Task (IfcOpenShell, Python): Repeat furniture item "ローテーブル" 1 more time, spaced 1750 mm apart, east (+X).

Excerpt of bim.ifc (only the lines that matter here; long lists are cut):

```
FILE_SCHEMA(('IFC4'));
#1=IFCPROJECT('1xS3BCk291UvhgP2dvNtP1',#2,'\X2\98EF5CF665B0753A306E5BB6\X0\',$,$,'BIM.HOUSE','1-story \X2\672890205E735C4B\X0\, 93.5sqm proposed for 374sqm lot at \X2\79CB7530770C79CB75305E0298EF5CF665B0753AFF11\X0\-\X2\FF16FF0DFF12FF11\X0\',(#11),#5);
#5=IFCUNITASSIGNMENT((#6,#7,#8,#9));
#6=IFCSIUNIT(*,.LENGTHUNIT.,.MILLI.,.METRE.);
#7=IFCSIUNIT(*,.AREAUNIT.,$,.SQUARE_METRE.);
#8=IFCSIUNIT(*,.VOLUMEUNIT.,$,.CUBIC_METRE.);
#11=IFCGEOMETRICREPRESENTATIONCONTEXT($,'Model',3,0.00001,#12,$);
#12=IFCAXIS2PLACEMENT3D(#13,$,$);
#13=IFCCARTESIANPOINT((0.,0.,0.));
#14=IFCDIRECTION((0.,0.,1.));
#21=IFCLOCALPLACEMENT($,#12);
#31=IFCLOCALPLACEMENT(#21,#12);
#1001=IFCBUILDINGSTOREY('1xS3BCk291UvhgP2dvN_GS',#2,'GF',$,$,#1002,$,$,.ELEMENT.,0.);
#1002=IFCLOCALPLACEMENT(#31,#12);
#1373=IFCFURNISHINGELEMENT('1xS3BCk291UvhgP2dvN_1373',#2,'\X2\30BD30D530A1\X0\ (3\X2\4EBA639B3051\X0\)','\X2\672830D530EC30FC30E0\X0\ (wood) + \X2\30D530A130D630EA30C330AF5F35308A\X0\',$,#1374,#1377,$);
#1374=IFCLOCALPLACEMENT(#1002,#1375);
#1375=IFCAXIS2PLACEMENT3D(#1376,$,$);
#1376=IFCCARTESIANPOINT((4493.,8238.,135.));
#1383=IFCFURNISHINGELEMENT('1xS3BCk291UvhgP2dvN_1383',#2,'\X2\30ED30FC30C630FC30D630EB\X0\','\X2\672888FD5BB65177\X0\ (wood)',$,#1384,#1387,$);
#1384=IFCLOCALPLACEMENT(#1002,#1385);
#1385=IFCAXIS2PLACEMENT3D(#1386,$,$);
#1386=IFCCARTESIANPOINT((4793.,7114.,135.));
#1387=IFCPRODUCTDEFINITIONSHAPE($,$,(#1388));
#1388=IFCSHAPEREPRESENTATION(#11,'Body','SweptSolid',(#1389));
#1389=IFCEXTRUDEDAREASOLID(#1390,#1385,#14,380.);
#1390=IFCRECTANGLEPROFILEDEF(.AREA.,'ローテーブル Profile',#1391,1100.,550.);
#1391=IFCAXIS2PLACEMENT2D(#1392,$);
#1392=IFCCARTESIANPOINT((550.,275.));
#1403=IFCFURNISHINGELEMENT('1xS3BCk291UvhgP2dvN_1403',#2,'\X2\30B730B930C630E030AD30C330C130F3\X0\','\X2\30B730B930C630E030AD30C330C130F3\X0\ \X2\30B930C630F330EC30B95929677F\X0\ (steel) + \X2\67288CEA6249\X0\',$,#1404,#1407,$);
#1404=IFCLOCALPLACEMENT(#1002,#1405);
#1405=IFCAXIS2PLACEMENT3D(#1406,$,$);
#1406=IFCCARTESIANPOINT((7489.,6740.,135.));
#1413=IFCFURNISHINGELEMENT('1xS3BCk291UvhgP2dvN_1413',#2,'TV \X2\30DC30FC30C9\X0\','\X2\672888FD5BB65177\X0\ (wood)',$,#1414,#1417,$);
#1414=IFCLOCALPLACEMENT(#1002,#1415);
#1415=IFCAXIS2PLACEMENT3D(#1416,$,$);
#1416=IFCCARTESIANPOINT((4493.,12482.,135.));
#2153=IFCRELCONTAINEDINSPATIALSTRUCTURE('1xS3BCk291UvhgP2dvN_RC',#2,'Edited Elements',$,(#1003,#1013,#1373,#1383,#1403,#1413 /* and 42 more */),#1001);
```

```python
import numpy as np
import ifcopenshell
import ifcopenshell.api.geometry
import ifcopenshell.api.root
import ifcopenshell.util.element
import ifcopenshell.util.placement
import ifcopenshell.util.unit

model = ifcopenshell.open("bim.ifc")
unit_scale = ifcopenshell.util.unit.calculate_unit_scale(model)


def reuse_history(source, copy):
    """copy_class also copies each property set's owner history, people and application; keep the originals."""
    for rel in copy.IsDefinedBy:
        if rel.is_a("IfcRelDefinesByProperties") and (history := rel.RelatingPropertyDefinition.OwnerHistory):
            rel.RelatingPropertyDefinition.OwnerHistory = source.OwnerHistory
            ifcopenshell.util.element.remove_deep2(model, history)


source = model.by_guid("1xS3BCk291UvhgP2dvN_1383")
base = ifcopenshell.util.placement.get_local_placement(source.ObjectPlacement)
step = np.array([1.0, 0.0, 0.0]) * 1.75 / unit_scale

for i in range(1, 2):
    copy = ifcopenshell.api.root.copy_class(model, product=source)
    copy.Representation = ifcopenshell.util.element.copy_deep(
        model, source.Representation, exclude=["IfcGeometricRepresentationContext", "IfcRepresentationMap"]
    )
    reuse_history(source, copy)
    matrix = base.copy()
    matrix[:3, 3] += i * step
    print("added at", matrix[:3, 3].round(3) + 0.0)
    ifcopenshell.api.geometry.edit_object_placement(model, product=copy, matrix=matrix, is_si=False)

model.write("bim_v2.ifc")
```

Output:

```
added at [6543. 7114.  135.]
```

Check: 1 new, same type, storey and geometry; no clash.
